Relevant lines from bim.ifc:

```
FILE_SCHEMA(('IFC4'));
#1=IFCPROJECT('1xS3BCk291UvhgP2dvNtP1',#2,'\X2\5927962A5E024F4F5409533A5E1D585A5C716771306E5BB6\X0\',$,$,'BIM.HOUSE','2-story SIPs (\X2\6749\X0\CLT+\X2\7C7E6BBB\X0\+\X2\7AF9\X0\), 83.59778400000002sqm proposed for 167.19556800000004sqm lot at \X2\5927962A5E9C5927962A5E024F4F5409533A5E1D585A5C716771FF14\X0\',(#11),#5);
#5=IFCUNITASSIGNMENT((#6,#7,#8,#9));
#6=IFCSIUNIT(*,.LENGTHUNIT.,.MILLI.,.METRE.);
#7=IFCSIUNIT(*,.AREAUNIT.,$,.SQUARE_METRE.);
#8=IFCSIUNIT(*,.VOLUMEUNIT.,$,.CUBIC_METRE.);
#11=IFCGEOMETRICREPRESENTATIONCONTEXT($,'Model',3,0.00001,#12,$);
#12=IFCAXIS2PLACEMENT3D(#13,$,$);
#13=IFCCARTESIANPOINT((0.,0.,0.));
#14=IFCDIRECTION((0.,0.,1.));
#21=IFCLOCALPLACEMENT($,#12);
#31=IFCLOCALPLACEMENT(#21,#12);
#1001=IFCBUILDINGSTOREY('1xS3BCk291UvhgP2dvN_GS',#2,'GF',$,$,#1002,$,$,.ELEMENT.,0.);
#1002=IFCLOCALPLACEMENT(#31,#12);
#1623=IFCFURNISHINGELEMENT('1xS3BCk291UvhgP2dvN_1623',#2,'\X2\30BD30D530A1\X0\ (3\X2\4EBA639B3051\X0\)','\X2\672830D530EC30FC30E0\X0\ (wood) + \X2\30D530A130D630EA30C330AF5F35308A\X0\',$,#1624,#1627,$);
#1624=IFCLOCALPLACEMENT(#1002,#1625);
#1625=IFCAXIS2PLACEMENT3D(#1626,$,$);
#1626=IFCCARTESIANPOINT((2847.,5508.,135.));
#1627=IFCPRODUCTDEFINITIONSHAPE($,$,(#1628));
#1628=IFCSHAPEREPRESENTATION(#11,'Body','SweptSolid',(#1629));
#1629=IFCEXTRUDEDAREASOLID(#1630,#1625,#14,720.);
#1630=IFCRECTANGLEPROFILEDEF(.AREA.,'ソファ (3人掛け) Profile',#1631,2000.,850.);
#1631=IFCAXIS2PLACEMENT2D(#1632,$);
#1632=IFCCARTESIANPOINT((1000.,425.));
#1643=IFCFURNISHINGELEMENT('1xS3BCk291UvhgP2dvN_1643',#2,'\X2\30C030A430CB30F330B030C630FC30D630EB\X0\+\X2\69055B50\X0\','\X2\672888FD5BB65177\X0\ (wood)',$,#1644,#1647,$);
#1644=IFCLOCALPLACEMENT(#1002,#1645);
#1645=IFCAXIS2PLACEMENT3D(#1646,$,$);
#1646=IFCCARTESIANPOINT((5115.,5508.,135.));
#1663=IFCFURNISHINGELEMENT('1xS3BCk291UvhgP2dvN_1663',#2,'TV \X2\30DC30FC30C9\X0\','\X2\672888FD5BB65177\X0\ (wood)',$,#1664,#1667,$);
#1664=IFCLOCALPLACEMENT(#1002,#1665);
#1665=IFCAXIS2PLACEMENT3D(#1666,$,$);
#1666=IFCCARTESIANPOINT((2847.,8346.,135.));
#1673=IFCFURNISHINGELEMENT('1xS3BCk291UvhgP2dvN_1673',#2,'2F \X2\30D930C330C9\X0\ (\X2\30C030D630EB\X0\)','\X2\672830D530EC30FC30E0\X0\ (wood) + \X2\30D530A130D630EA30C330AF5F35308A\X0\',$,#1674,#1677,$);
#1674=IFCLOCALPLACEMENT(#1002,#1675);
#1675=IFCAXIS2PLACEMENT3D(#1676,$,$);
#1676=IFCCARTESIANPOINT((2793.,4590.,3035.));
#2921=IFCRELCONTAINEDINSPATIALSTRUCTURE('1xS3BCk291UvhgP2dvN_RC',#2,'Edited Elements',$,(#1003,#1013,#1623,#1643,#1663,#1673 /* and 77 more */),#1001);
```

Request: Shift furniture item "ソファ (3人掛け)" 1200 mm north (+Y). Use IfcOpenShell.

```python
import ifcopenshell
import ifcopenshell.api.geometry
import ifcopenshell.util.placement
import ifcopenshell.util.unit

model = ifcopenshell.open("bim.ifc")
unit_scale = ifcopenshell.util.unit.calculate_unit_scale(model)

item = model.by_guid("1xS3BCk291UvhgP2dvN_1623")
matrix = ifcopenshell.util.placement.get_local_placement(item.ObjectPlacement)
matrix[1, 3] += 1.2 / unit_scale
ifcopenshell.api.geometry.edit_object_placement(model, product=item, matrix=matrix, is_si=False)

print(ifcopenshell.util.placement.get_local_placement(item.ObjectPlacement).round(3) + 0.0)

model.write("bim_rev.ifc")
```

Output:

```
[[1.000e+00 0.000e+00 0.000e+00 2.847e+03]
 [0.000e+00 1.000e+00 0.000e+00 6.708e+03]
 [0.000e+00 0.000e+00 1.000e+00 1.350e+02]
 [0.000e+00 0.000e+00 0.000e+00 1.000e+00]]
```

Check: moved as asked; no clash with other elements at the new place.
